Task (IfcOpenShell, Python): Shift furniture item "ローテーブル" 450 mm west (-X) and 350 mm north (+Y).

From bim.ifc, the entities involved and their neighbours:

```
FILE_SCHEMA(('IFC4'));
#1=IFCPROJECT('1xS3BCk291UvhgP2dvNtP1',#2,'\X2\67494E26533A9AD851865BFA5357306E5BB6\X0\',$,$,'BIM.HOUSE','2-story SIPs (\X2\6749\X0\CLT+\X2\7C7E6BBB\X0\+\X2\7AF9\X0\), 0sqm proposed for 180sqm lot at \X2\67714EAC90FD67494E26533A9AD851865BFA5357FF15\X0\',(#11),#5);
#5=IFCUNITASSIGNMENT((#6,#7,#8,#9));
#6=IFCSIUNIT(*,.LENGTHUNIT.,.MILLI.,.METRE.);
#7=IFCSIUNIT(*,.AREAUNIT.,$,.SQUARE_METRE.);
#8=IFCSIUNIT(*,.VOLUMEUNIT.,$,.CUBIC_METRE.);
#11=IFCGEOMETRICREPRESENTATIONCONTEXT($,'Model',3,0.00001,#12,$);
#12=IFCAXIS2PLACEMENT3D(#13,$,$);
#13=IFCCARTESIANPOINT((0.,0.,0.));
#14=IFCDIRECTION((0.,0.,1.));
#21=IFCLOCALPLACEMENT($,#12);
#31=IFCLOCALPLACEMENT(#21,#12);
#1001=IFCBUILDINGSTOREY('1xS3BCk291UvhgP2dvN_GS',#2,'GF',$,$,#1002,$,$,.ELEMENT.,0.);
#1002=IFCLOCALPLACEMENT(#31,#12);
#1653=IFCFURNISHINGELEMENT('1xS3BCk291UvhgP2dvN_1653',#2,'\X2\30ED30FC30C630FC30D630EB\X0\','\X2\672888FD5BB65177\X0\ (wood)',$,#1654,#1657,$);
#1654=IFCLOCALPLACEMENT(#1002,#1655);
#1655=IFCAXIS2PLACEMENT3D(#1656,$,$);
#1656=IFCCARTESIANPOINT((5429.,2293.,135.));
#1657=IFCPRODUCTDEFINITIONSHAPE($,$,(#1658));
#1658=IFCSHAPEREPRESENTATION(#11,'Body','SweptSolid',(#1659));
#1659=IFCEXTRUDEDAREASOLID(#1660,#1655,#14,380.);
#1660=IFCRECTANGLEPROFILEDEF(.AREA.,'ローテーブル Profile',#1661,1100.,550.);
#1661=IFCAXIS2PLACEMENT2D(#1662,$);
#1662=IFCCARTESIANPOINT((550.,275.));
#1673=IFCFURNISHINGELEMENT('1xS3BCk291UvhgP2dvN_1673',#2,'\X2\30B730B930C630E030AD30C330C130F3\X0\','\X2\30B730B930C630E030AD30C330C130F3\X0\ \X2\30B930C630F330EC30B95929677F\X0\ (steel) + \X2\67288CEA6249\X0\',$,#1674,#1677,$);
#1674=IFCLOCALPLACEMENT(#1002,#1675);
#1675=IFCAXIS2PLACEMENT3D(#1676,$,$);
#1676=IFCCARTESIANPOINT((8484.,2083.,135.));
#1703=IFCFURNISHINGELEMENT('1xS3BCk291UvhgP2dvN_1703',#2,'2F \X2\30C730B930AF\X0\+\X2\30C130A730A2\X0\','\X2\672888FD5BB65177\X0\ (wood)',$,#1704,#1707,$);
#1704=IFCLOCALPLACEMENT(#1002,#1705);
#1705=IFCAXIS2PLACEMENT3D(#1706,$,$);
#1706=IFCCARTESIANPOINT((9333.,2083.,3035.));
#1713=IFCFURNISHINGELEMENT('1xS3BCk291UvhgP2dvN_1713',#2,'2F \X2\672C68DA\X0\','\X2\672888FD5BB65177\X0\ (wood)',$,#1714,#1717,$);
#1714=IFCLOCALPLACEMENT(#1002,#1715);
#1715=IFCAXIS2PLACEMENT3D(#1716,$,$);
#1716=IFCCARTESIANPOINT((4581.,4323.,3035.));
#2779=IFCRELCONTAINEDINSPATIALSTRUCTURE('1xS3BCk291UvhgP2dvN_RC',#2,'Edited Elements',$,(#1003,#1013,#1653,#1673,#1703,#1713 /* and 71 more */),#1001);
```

```python
import ifcopenshell
import ifcopenshell.api.geometry
import ifcopenshell.util.placement
import ifcopenshell.util.unit

model = ifcopenshell.open("bim.ifc")
unit_scale = ifcopenshell.util.unit.calculate_unit_scale(model)

item = model.by_guid("1xS3BCk291UvhgP2dvN_1653")
matrix = ifcopenshell.util.placement.get_local_placement(item.ObjectPlacement)
matrix[0, 3] -= 0.45 / unit_scale
matrix[1, 3] += 0.35 / unit_scale
ifcopenshell.api.geometry.edit_object_placement(model, product=item, matrix=matrix, is_si=False)

print(ifcopenshell.util.placement.get_local_placement(item.ObjectPlacement).round(3) + 0.0)

model.write("bim_v2.ifc")
```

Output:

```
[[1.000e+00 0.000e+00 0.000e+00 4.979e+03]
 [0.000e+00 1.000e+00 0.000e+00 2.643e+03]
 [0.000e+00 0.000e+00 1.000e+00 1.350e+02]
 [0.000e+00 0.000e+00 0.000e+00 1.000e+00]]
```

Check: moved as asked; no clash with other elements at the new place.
